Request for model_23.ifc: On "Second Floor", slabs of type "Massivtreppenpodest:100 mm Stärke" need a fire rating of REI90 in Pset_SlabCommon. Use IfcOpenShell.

First a look at what the model holds.

```python
import ifcopenshell
import ifcopenshell.util.element

model = ifcopenshell.open("model_23.ifc")
print(model.schema)
storey = next(s for s in model.by_type("IfcBuildingStorey") if s.Name == "Second Floor")
slabs = [e for e in ifcopenshell.util.element.get_decomposition(storey) if e.is_a("IfcSlab")]
seen = {}
for e in slabs:
    element_type = ifcopenshell.util.element.get_type(e)
    key = (element_type.Name if element_type != e and element_type else None, ifcopenshell.util.element.get_pset(e, "Pset_SlabCommon", "FireRating"))
    seen[key] = seen.get(key, 0) + 1
for (name, value), count in sorted(seen.items(), key=str):
    print(count, "x", name, "|", value)
```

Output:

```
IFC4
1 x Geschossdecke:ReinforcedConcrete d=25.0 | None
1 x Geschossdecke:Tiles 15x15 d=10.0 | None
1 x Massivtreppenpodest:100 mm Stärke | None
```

```python
import ifcopenshell
import ifcopenshell.api.pset
import ifcopenshell.util.element

model = ifcopenshell.open("model_23.ifc")

storey = next(s for s in model.by_type("IfcBuildingStorey") if s.Name == "Second Floor")
slabs = [e for e in ifcopenshell.util.element.get_decomposition(storey) if e.is_a("IfcSlab")]

count = 0
for e in slabs:
    element_type = ifcopenshell.util.element.get_type(e)
    if element_type in (None, e) or element_type.Name != "Massivtreppenpodest:100 mm Stärke":
        continue
    # add_pset returns the element's existing set when there is one.
    pset = ifcopenshell.api.pset.add_pset(model, product=e, name="Pset_SlabCommon")
    ifcopenshell.api.pset.edit_pset(model, pset=pset, properties={"FireRating": "REI90"})
    count += 1

print(count, "slabs updated")

model.write("model_23_updated.ifc")
```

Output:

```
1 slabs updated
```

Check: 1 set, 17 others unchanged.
